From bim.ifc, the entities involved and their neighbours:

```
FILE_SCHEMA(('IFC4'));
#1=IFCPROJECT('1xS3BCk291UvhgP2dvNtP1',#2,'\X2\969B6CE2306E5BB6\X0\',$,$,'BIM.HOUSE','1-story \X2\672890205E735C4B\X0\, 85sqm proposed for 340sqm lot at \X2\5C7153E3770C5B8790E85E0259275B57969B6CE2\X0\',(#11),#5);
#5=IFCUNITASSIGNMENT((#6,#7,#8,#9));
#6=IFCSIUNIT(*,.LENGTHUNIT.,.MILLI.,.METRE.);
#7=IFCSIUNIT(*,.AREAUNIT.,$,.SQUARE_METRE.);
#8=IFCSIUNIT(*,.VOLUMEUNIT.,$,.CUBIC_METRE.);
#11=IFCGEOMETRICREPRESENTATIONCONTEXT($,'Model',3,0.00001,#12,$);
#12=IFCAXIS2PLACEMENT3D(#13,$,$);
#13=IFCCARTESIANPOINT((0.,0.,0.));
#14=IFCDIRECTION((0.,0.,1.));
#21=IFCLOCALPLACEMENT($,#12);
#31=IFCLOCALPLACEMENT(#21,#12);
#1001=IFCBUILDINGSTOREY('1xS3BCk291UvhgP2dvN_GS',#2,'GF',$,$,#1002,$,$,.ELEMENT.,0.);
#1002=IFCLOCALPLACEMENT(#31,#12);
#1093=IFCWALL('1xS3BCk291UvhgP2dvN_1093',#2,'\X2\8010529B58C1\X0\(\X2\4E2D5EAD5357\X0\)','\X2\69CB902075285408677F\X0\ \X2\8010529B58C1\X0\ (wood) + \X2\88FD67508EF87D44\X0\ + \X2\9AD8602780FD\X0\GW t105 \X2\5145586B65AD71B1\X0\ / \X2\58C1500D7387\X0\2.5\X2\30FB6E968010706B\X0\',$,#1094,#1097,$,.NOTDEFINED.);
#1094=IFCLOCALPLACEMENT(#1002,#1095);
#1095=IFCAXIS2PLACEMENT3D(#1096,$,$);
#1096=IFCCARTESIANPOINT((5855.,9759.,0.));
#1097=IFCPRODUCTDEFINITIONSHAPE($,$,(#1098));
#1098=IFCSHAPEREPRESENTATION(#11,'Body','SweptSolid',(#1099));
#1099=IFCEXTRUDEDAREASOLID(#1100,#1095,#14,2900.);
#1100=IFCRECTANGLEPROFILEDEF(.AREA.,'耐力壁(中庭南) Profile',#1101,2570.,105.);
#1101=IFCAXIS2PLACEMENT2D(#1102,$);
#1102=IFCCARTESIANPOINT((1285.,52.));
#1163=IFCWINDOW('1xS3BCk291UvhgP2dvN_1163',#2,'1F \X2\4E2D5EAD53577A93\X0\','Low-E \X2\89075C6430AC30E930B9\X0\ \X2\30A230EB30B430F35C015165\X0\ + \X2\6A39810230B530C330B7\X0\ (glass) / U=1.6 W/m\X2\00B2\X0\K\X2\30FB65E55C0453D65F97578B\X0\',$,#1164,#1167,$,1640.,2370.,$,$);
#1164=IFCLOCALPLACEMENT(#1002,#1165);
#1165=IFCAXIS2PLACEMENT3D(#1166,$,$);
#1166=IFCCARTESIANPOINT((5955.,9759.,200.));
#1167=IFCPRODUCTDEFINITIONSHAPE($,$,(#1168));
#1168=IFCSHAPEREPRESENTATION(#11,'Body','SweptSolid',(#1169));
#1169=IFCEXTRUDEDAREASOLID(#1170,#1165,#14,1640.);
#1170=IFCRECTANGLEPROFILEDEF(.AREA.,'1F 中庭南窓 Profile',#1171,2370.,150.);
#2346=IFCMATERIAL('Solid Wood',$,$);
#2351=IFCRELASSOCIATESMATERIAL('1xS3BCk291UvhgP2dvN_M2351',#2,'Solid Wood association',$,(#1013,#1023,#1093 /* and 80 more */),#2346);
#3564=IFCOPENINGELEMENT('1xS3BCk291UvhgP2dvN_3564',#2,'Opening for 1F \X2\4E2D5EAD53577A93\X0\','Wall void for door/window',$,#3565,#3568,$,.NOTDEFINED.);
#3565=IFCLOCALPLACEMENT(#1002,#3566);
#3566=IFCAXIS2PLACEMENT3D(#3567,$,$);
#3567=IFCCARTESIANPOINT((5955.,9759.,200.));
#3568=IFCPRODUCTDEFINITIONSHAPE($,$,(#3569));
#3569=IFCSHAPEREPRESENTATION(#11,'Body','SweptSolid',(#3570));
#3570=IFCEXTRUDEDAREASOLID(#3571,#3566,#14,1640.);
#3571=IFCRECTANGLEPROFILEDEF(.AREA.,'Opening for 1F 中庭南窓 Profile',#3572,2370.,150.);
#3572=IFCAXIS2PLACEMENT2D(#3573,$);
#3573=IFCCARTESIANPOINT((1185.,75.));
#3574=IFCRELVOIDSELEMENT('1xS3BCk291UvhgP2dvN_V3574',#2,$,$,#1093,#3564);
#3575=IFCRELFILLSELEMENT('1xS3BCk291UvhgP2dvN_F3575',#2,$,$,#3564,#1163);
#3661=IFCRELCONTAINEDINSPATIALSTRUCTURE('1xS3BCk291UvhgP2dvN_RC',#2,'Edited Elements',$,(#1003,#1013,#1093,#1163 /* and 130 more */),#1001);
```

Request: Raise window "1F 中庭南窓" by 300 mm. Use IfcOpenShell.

```python
import numpy as np
import ifcopenshell
import ifcopenshell.api.geometry
import ifcopenshell.util.placement
import ifcopenshell.util.unit

model = ifcopenshell.open("bim.ifc")
unit_scale = ifcopenshell.util.unit.calculate_unit_scale(model)

window = model.by_guid("1xS3BCk291UvhgP2dvN_1163")
opening = window.FillsVoids[0].RelatingOpeningElement
dz = 0.3 / unit_scale

shift = np.array([0.0, 0.0, dz])
# The window is not placed relative to its opening, so move both.
for product in (opening, window):
    matrix = ifcopenshell.util.placement.get_local_placement(product.ObjectPlacement)
    matrix[:3, 3] += shift
    ifcopenshell.api.geometry.edit_object_placement(model, product=product, matrix=matrix, is_si=False)

print(f"moved by {dz * unit_scale:+.3f} m")

model.write("bim_v2.ifc")
```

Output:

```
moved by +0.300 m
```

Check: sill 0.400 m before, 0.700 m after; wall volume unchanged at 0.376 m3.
